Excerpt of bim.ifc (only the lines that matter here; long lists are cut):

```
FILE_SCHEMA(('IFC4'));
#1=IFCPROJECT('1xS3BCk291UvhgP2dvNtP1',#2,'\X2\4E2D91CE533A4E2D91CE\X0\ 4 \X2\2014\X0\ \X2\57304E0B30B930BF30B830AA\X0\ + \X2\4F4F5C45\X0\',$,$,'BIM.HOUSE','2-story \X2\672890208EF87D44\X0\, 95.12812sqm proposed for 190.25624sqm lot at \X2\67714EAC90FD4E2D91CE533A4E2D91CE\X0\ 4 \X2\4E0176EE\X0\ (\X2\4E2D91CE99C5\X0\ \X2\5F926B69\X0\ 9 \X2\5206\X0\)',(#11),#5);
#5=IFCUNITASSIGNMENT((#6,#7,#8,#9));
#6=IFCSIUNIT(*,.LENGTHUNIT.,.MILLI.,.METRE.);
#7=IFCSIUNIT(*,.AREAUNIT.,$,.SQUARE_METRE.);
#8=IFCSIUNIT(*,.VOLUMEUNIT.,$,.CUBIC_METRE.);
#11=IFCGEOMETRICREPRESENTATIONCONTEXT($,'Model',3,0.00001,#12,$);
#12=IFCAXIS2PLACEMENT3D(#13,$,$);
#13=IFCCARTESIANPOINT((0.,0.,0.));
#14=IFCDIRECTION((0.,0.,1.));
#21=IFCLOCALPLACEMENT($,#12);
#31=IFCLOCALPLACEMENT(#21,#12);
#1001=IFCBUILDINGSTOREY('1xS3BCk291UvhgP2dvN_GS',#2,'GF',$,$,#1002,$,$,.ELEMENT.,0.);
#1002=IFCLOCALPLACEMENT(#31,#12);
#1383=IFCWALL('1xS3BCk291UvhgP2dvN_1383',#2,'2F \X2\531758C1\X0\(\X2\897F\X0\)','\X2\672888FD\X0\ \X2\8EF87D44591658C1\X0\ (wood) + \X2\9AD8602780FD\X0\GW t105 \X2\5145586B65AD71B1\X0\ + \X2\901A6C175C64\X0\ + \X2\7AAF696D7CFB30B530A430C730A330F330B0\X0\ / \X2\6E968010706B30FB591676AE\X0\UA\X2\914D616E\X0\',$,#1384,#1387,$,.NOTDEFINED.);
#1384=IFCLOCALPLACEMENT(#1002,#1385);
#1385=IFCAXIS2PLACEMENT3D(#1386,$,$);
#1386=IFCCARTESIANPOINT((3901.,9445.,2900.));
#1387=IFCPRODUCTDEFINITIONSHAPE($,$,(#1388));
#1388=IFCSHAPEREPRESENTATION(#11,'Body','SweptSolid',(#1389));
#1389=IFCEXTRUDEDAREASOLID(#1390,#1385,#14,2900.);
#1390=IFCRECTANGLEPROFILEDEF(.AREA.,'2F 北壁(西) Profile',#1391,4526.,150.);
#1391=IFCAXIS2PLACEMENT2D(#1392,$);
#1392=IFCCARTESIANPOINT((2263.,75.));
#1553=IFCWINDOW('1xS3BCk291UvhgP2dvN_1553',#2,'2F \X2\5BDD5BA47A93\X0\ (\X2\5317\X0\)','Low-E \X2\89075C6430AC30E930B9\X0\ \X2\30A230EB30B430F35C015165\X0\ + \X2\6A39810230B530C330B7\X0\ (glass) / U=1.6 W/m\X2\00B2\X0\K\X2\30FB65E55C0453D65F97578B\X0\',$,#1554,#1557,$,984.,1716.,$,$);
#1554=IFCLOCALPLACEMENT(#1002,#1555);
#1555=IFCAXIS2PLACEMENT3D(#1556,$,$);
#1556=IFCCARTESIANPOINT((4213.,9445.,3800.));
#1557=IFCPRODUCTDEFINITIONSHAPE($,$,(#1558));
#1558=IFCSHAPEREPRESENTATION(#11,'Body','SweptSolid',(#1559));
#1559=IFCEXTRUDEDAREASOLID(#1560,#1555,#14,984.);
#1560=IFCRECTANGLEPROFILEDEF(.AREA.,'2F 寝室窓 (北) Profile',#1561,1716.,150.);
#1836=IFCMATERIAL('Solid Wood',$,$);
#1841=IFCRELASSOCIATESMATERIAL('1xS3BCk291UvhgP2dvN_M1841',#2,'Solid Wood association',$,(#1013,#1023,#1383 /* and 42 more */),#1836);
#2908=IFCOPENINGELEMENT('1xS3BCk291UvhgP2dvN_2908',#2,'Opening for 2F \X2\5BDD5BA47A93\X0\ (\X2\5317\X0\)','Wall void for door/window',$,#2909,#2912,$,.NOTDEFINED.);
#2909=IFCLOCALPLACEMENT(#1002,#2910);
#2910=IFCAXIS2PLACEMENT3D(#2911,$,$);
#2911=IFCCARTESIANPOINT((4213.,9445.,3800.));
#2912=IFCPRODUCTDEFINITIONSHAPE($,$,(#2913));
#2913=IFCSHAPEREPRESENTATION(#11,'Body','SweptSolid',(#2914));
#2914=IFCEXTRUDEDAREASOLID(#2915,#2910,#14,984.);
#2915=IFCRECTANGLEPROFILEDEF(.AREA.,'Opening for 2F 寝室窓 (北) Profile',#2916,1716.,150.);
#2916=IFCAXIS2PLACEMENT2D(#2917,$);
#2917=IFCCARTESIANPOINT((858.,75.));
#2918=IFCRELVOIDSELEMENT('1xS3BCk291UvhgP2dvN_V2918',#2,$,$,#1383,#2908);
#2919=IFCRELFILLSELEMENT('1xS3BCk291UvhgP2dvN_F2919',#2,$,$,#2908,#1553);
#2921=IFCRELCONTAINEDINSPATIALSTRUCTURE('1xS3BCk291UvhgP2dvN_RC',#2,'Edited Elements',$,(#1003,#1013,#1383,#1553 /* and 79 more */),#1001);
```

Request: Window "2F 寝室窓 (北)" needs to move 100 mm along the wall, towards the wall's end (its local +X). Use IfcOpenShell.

```python
import ifcopenshell
import ifcopenshell.api.geometry
import ifcopenshell.util.placement
import ifcopenshell.util.unit

model = ifcopenshell.open("bim.ifc")
unit_scale = ifcopenshell.util.unit.calculate_unit_scale(model)

window = model.by_id(1553)
opening = window.FillsVoids[0].RelatingOpeningElement
wall = opening.VoidsElements[0].RelatingBuildingElement

wall_matrix = ifcopenshell.util.placement.get_local_placement(wall.ObjectPlacement)
shift = wall_matrix[:3, 0] * 0.1 / unit_scale
before = ifcopenshell.util.placement.get_local_placement(window.ObjectPlacement)[:3, 3].copy()

# The window is not placed relative to its opening, so move both.
for product in (opening, window):
    matrix = ifcopenshell.util.placement.get_local_placement(product.ObjectPlacement)
    matrix[:3, 3] += shift
    ifcopenshell.api.geometry.edit_object_placement(model, product=product, matrix=matrix, is_si=False)

after = ifcopenshell.util.placement.get_local_placement(window.ObjectPlacement)[:3, 3]
print("window moved by", (after - before).round(3) + 0.0)

model.write("bim-out.ifc")
```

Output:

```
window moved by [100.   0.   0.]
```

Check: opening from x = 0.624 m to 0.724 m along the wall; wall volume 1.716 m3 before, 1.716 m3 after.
